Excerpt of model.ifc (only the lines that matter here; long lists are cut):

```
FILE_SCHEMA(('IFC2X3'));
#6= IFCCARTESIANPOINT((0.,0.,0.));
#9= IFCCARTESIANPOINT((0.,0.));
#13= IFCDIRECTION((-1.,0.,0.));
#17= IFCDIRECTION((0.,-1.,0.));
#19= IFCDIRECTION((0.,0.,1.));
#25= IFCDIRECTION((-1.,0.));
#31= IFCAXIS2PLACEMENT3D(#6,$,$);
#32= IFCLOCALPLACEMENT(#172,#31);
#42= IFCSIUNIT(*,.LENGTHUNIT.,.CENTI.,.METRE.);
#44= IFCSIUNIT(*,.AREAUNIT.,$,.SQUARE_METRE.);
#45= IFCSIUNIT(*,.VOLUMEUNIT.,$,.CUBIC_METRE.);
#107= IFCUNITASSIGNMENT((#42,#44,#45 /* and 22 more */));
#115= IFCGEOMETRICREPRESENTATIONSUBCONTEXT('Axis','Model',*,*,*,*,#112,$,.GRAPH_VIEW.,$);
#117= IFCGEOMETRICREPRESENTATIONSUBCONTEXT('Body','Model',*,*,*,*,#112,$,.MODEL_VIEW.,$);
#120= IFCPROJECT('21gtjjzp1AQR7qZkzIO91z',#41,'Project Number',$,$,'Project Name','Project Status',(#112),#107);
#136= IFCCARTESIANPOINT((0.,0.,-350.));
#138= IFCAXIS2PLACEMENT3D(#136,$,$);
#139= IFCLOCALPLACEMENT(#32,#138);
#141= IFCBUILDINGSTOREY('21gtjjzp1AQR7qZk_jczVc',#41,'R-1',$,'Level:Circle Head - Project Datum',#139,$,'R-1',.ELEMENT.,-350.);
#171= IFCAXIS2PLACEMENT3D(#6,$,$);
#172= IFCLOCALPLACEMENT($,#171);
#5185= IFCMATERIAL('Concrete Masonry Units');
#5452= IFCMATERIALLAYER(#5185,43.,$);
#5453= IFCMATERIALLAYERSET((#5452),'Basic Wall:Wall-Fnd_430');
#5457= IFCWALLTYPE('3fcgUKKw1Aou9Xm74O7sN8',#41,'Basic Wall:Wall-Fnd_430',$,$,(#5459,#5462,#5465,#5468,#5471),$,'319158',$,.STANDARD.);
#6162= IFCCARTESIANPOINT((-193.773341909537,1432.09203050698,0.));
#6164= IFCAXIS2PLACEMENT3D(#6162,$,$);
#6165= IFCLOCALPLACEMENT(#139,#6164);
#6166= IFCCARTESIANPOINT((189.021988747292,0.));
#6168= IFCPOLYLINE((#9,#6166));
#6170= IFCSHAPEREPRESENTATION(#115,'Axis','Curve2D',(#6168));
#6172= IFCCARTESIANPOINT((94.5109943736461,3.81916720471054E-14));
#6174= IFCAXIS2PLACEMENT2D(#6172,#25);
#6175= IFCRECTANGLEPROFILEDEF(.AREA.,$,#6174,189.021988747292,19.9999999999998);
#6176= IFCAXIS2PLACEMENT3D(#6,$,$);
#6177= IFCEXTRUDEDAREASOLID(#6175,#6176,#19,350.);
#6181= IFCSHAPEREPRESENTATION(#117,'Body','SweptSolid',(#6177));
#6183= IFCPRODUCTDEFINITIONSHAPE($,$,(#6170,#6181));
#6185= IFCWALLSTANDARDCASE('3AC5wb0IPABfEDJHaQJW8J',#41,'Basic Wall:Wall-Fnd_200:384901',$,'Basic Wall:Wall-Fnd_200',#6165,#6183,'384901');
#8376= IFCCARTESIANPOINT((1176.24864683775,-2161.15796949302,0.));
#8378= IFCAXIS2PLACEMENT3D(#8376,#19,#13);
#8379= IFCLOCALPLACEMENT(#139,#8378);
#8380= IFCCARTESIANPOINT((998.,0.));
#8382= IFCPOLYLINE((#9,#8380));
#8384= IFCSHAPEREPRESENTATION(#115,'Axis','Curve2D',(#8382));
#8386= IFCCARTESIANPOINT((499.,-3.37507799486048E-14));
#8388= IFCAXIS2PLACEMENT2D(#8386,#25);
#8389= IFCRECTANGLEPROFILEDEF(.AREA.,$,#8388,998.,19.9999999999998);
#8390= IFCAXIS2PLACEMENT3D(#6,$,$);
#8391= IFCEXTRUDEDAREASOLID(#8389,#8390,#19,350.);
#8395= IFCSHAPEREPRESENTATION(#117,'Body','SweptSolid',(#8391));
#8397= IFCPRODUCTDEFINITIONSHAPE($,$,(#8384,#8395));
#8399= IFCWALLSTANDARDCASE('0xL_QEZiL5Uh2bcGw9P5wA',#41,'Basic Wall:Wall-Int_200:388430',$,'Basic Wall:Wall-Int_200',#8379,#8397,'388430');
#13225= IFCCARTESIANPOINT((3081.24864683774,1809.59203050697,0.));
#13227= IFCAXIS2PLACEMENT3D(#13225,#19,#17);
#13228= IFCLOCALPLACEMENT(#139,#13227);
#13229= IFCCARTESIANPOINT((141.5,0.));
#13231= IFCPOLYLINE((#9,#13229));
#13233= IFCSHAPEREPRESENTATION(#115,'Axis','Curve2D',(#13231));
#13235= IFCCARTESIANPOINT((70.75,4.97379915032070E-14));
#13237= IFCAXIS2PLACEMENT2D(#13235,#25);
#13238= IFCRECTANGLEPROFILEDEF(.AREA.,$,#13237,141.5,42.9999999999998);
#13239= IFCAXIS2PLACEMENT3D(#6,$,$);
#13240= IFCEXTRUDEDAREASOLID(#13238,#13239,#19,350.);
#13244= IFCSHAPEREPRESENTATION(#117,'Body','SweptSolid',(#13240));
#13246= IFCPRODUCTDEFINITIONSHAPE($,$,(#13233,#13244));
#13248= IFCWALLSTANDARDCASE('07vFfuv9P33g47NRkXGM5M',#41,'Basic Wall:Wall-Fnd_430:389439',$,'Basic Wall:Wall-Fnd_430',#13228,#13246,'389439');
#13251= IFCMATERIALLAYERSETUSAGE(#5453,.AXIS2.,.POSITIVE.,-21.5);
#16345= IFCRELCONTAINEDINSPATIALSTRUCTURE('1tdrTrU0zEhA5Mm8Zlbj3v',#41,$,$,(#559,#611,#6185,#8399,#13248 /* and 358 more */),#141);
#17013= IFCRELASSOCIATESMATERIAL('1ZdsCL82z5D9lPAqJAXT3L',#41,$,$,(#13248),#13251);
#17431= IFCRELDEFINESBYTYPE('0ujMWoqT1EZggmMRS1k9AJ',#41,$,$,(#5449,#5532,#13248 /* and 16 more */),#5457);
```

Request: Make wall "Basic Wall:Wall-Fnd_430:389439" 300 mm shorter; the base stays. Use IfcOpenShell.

```python
import ifcopenshell
import ifcopenshell.geom
import ifcopenshell.util.representation
import ifcopenshell.util.shape
import ifcopenshell.util.unit

model = ifcopenshell.open("model.ifc")
unit_scale = ifcopenshell.util.unit.calculate_unit_scale(model)
settings = ifcopenshell.geom.settings()


def volume(element):
    """Net volume in cubic metres, openings subtracted."""
    shape = ifcopenshell.geom.create_shape(settings, element)
    return ifcopenshell.util.shape.get_volume(shape.geometry)


wall = model.by_id(13248)
before = volume(wall)

body = ifcopenshell.util.representation.get_representation(wall, "Model", "Body")
solid = body.Items[0]
old_height = solid.Depth
solid.Depth -= 0.3 / unit_scale
after = volume(wall)

print(f"height {old_height:g} -> {solid.Depth:g}, volume {before:.3f} -> {after:.3f} m3")

model.write("model_updated.ifc")
```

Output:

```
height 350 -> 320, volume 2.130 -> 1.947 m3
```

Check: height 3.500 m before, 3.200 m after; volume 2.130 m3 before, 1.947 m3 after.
